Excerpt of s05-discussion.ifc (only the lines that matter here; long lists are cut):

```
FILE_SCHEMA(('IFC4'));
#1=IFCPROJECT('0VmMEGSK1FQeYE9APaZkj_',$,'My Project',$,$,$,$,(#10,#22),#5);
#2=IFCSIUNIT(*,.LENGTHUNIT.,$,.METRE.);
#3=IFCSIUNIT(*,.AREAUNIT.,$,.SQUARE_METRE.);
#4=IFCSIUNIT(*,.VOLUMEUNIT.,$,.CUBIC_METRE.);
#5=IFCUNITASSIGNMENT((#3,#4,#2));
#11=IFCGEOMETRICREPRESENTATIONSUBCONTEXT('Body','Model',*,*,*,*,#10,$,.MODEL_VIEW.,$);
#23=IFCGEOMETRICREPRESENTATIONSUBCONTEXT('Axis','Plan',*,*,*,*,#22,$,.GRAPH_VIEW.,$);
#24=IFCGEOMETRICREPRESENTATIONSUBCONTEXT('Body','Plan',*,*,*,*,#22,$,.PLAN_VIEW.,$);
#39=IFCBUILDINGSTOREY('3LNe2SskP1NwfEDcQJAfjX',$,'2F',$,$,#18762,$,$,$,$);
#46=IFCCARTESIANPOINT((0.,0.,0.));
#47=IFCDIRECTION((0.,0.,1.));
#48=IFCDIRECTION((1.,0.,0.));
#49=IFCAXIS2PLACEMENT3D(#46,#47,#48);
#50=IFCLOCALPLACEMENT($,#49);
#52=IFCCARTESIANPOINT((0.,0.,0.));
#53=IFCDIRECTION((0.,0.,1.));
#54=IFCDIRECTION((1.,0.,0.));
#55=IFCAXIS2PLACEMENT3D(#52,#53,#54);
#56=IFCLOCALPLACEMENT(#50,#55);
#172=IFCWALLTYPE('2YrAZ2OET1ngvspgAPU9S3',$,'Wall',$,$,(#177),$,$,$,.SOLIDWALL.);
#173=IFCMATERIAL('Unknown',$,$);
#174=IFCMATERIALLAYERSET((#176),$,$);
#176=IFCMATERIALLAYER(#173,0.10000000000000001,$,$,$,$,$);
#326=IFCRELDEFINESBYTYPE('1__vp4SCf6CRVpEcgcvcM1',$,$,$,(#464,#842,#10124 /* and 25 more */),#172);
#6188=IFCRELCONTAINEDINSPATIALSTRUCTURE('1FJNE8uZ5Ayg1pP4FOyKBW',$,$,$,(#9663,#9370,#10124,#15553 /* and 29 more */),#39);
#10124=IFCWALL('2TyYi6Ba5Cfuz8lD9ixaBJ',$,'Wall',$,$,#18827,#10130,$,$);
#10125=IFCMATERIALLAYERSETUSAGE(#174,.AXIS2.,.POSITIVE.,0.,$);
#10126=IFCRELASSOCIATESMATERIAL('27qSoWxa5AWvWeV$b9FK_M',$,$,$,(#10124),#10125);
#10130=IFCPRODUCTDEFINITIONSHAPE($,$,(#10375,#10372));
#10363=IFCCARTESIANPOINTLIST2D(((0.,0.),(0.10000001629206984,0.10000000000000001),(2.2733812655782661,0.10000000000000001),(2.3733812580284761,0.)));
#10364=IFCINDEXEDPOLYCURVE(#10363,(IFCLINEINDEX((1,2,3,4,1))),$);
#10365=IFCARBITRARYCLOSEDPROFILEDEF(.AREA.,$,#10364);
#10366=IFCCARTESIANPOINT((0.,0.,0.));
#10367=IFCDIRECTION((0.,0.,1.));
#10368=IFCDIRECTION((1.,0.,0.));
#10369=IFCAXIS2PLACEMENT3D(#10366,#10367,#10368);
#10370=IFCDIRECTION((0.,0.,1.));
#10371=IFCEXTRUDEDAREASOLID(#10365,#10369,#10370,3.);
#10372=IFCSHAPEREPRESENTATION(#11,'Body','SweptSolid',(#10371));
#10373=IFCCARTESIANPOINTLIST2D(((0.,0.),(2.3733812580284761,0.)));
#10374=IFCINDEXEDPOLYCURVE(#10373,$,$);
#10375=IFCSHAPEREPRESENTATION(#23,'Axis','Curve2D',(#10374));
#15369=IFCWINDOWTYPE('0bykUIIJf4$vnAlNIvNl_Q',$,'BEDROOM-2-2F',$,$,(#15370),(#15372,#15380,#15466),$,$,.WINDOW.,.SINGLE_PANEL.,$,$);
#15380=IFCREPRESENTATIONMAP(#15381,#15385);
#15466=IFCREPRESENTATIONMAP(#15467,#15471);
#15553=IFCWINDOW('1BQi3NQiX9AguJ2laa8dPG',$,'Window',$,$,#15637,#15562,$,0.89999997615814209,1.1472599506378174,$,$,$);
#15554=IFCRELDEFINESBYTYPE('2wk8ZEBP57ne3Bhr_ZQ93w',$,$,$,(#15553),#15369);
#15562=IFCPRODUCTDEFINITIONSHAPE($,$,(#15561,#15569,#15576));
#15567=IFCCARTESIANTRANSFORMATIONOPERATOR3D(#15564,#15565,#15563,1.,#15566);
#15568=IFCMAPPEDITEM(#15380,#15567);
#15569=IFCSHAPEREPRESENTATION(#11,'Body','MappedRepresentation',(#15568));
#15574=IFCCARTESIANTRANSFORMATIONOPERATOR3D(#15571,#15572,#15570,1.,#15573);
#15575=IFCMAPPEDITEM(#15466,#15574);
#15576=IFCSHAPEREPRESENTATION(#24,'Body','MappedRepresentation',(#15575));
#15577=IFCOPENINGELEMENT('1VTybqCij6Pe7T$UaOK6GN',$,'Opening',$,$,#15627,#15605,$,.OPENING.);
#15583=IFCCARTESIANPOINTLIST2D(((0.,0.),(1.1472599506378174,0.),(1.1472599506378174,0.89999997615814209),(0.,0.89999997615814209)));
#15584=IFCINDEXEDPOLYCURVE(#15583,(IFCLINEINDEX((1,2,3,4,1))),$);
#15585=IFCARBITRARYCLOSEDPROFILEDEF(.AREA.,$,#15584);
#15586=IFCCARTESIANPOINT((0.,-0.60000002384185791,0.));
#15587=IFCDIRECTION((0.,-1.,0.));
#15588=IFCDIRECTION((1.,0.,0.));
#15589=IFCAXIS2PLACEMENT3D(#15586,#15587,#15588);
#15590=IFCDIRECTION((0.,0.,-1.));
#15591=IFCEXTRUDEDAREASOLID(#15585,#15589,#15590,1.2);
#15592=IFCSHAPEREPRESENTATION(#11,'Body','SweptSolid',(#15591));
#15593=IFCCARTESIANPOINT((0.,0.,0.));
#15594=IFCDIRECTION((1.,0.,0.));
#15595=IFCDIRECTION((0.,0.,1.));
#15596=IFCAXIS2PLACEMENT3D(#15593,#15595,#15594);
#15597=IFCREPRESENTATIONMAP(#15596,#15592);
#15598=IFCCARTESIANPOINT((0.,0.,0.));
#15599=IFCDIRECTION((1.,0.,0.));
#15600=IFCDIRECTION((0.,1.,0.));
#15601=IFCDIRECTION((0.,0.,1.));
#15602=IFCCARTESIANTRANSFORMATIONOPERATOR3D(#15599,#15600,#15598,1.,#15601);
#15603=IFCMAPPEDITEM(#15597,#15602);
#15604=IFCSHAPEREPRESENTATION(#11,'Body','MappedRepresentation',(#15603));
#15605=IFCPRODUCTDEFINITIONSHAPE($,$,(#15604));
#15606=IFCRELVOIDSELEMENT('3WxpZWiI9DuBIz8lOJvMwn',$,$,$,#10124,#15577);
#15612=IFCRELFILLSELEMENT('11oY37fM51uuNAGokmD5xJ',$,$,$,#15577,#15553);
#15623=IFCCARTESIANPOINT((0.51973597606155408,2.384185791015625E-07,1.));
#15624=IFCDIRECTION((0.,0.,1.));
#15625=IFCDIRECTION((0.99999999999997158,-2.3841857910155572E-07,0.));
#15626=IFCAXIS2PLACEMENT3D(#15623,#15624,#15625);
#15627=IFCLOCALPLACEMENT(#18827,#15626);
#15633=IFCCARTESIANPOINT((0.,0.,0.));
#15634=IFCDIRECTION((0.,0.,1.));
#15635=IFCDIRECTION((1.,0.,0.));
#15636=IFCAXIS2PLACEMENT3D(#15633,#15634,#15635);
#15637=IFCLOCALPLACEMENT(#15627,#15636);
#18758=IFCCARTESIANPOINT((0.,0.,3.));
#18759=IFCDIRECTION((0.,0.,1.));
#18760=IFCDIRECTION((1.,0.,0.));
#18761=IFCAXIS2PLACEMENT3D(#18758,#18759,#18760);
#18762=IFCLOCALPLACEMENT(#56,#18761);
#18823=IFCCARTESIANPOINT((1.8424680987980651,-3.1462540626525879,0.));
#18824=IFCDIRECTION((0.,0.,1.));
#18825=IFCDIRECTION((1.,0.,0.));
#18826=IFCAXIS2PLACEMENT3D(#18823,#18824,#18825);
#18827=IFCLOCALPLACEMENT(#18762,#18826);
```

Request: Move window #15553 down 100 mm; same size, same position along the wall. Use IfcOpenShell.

```python
import numpy as np
import ifcopenshell
import ifcopenshell.api.geometry
import ifcopenshell.util.placement
import ifcopenshell.util.unit

model = ifcopenshell.open("s05-discussion.ifc")
unit_scale = ifcopenshell.util.unit.calculate_unit_scale(model)

window = model.by_guid("1BQi3NQiX9AguJ2laa8dPG")
opening = window.FillsVoids[0].RelatingOpeningElement
dz = -0.1

shift = np.array([0.0, 0.0, dz])
# The window is placed relative to its opening, so it follows when the opening moves.
matrix = ifcopenshell.util.placement.get_local_placement(opening.ObjectPlacement)
matrix[:3, 3] += shift
ifcopenshell.api.geometry.edit_object_placement(
    model, product=opening, matrix=matrix, is_si=False, should_transform_children=True
)

print(f"moved by {dz * unit_scale:+.3f} m")

model.write("s05-discussion_updated.ifc")
```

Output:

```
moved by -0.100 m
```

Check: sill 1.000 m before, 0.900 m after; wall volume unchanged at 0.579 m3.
